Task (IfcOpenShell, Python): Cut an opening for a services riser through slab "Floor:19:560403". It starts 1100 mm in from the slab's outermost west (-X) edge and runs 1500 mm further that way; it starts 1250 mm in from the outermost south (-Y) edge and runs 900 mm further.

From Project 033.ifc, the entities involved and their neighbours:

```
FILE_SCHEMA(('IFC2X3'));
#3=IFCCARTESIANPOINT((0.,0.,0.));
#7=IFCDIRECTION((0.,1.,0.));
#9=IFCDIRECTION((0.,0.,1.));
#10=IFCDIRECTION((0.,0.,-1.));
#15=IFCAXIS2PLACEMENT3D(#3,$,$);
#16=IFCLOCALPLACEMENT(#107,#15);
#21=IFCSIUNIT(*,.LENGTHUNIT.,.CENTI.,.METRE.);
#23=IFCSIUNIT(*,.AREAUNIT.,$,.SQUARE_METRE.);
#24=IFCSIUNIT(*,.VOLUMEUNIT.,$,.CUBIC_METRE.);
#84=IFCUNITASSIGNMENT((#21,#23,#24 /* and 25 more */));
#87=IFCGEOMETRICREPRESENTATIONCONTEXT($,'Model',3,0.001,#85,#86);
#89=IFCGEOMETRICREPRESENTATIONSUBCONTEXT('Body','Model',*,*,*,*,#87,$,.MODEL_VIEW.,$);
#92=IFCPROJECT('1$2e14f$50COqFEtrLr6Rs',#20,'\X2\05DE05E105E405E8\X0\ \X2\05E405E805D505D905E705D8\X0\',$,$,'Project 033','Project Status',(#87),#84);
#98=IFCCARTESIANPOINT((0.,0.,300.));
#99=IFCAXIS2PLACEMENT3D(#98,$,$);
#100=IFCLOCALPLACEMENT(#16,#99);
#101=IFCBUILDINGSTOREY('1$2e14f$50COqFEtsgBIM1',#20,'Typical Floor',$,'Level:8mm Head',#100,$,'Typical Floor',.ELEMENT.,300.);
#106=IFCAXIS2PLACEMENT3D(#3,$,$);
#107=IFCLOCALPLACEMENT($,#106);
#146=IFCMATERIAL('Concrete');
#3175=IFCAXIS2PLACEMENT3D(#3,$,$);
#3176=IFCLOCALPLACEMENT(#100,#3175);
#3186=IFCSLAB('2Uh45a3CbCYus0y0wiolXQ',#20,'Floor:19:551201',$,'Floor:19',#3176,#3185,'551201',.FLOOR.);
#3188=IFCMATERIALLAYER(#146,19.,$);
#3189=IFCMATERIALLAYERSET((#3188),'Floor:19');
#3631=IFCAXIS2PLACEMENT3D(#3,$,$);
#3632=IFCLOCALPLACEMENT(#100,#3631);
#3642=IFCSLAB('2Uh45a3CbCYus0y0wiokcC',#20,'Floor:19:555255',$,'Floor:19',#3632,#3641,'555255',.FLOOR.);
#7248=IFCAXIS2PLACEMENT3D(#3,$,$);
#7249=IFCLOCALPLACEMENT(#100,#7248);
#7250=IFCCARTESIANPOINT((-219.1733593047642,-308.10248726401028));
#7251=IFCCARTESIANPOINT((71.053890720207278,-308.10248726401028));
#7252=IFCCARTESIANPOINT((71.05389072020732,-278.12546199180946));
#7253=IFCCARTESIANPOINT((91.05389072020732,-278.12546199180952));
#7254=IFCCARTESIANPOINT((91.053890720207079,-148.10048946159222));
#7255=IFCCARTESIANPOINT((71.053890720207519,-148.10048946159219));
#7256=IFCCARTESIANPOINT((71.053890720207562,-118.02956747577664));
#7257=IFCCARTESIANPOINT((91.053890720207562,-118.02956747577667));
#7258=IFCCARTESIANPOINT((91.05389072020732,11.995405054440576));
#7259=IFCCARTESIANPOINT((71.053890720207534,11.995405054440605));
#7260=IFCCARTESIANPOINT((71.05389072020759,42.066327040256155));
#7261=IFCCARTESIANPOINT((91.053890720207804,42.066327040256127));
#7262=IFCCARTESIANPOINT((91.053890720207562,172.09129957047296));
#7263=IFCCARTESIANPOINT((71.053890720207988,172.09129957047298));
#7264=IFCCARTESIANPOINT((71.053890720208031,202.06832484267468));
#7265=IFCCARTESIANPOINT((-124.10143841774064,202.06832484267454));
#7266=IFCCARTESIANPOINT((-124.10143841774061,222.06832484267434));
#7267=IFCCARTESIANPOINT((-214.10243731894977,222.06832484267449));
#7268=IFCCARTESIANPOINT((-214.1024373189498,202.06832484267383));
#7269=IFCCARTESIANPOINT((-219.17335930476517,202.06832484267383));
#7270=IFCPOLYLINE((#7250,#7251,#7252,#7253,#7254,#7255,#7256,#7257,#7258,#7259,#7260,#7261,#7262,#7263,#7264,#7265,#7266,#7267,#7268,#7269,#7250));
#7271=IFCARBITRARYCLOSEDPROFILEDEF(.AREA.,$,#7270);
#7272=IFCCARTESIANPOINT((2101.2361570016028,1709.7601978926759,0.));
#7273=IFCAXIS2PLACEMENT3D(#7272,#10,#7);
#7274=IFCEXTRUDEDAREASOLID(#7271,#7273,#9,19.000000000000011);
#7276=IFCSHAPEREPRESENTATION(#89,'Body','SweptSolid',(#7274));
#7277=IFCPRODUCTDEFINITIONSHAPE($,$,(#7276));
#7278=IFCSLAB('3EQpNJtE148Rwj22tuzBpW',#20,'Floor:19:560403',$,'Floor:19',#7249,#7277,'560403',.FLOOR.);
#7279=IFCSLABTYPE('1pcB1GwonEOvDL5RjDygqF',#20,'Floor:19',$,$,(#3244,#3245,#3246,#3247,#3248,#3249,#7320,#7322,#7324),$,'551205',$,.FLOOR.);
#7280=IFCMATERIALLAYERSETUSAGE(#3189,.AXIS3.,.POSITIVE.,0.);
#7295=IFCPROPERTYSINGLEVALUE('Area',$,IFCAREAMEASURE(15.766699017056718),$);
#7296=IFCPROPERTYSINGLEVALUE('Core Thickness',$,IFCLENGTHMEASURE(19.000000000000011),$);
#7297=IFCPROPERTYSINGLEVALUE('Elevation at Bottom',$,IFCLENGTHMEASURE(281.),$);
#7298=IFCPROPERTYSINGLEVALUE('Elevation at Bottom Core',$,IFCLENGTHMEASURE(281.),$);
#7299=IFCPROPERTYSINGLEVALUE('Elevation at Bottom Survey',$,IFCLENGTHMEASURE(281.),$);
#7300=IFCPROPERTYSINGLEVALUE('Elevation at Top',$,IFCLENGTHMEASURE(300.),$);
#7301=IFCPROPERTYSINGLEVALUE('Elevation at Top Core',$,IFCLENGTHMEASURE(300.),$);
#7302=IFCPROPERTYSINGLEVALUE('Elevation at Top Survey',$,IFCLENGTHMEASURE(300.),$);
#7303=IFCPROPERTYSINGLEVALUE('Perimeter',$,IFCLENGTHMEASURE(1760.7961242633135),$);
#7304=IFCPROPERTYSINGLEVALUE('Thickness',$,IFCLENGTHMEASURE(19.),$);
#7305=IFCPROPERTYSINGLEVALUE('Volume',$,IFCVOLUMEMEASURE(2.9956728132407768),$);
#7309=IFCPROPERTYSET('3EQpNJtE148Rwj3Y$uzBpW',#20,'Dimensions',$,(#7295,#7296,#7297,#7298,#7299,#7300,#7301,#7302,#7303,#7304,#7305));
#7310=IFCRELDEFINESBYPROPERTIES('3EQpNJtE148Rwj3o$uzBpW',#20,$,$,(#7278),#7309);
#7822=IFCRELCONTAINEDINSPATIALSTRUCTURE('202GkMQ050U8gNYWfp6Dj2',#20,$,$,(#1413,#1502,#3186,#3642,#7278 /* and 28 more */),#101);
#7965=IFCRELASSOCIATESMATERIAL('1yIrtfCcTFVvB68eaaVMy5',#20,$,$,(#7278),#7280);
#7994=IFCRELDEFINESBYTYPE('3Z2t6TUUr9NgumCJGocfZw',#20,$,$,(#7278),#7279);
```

```python
import numpy as np
import ifcopenshell
import ifcopenshell.api.feature
import ifcopenshell.api.geometry
import ifcopenshell.api.pset
import ifcopenshell.api.root
import ifcopenshell.geom
import ifcopenshell.util.element
import ifcopenshell.util.placement
import ifcopenshell.util.representation
import ifcopenshell.util.shape
import ifcopenshell.util.unit

model = ifcopenshell.open("Project 033.ifc")
unit_scale = ifcopenshell.util.unit.calculate_unit_scale(model)
area_scale = ifcopenshell.util.unit.calculate_unit_scale(model, "AREAUNIT")
volume_scale = ifcopenshell.util.unit.calculate_unit_scale(model, "VOLUMEUNIT")
settings = ifcopenshell.geom.settings()


def volume(element):
    """Net volume in cubic metres, openings subtracted."""
    shape = ifcopenshell.geom.create_shape(settings, element)
    return ifcopenshell.util.shape.get_volume(shape.geometry)


slab = model.by_id(7278)
before = volume(slab)

# Extent in the slab's own axes, in metres. The edges named are its -X and -Y sides.
slab_shape = ifcopenshell.geom.create_shape(settings, slab)
vertices = ifcopenshell.util.shape.get_vertices(slab_shape.geometry)
x_min, y_min, bottom = vertices.min(axis=0)
top = vertices[:, 2].max()

opening = ifcopenshell.api.root.create_entity(model, ifc_class="IfcOpeningElement", name="Services riser opening")
context = ifcopenshell.util.representation.get_context(model, "Model", "Body", "MODEL_VIEW")
width, depth = 1.5, 0.9
outline = [(0.0, 0.0), (width, 0.0), (width, depth), (0.0, depth), (0.0, 0.0)]
# Overshoot both faces by 50 mm so the cut is clean.
shape = ifcopenshell.api.geometry.add_slab_representation(
    model, context=context, depth=top - bottom + 0.1, polyline=outline
)
ifcopenshell.api.geometry.assign_representation(model, product=opening, representation=shape)

matrix = ifcopenshell.util.placement.get_local_placement(slab.ObjectPlacement)
matrix[:, 3] = matrix @ np.append(np.array([x_min + 1.1, y_min + 1.25, bottom - 0.05]) / unit_scale, 1.0)
ifcopenshell.api.geometry.edit_object_placement(model, product=opening, matrix=matrix, is_si=False)
ifcopenshell.api.feature.add_feature(model, feature=opening, element=slab)

after = volume(slab)

# Update the slab's stored quantities.
pset = model.by_id(ifcopenshell.util.element.get_pset(slab, "Dimensions", should_inherit=False)["id"])
ifcopenshell.api.pset.edit_pset(model, pset=pset, properties={
    "Area": model.create_entity("IfcAreaMeasure", after / (top - bottom) / area_scale),
    "Volume": model.create_entity("IfcVolumeMeasure", after / volume_scale),
})

print(f"slab volume {before:.3f} -> {after:.3f} m3")

model.write("Project 033_v2.ifc")
```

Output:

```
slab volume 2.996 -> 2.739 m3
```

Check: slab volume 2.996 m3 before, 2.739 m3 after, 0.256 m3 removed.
